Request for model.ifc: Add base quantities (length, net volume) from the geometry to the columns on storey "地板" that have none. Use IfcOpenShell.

First a look at what the model holds.

```python
import ifcopenshell
import ifcopenshell.util.element
import ifcopenshell.util.unit

model = ifcopenshell.open("model.ifc")
print(model.schema)
for unit_type in ("LENGTHUNIT", "AREAUNIT", "VOLUMEUNIT"):
    print(unit_type, ifcopenshell.util.unit.calculate_unit_scale(model, unit_type))
storey = next(s for s in model.by_type("IfcBuildingStorey") if s.Name == "地板")
columns = [e for e in ifcopenshell.util.element.get_decomposition(storey) if e.is_a("IfcColumn")]
for e in sorted(columns, key=lambda e: e.id()):
    print(e.id(), e.is_a(), e.Name, list(ifcopenshell.util.element.get_psets(e, qtos_only=True)), sep=" | ")
```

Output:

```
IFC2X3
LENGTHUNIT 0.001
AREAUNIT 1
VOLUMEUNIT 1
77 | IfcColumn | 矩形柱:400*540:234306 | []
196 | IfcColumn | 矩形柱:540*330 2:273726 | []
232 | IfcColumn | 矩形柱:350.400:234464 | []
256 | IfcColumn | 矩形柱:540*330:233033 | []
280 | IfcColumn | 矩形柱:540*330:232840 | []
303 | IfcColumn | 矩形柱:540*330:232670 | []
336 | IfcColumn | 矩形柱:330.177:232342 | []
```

```python
import ifcopenshell
import ifcopenshell.api.pset
import ifcopenshell.geom
import ifcopenshell.util.element
import ifcopenshell.util.shape
import ifcopenshell.util.unit

model = ifcopenshell.open("model.ifc")
unit_scale = ifcopenshell.util.unit.calculate_unit_scale(model)
volume_scale = ifcopenshell.util.unit.calculate_unit_scale(model, "VOLUMEUNIT")
settings = ifcopenshell.geom.settings()

storey = next(s for s in model.by_type("IfcBuildingStorey") if s.Name == "地板")
columns = [e for e in ifcopenshell.util.element.get_decomposition(storey) if e.is_a("IfcColumn")]

for e in sorted(columns, key=lambda e: e.id()):
    if ifcopenshell.util.element.get_psets(e, qtos_only=True, should_inherit=False):
        continue
    # Geometry comes back in metres, in the element's own axes.
    shape = ifcopenshell.geom.create_shape(settings, e)
    values = {
        "Length": ifcopenshell.util.shape.get_z(shape.geometry) / unit_scale,
        "NetVolume": ifcopenshell.util.shape.get_volume(shape.geometry) / volume_scale,
    }
    qto = ifcopenshell.api.pset.add_qto(model, product=e, name="BaseQuantities")
    ifcopenshell.api.pset.edit_qto(model, qto=qto, properties=values)
    print(e.id(), {k: round(v, 3) for k, v in values.items()})

model.write("model-out.ifc")
```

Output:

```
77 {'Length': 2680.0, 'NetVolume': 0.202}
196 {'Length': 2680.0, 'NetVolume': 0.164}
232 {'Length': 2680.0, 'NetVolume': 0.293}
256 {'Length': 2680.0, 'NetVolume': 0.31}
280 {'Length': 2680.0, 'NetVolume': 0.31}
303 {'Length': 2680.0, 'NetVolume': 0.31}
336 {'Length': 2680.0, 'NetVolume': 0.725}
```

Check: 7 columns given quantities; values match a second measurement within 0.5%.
